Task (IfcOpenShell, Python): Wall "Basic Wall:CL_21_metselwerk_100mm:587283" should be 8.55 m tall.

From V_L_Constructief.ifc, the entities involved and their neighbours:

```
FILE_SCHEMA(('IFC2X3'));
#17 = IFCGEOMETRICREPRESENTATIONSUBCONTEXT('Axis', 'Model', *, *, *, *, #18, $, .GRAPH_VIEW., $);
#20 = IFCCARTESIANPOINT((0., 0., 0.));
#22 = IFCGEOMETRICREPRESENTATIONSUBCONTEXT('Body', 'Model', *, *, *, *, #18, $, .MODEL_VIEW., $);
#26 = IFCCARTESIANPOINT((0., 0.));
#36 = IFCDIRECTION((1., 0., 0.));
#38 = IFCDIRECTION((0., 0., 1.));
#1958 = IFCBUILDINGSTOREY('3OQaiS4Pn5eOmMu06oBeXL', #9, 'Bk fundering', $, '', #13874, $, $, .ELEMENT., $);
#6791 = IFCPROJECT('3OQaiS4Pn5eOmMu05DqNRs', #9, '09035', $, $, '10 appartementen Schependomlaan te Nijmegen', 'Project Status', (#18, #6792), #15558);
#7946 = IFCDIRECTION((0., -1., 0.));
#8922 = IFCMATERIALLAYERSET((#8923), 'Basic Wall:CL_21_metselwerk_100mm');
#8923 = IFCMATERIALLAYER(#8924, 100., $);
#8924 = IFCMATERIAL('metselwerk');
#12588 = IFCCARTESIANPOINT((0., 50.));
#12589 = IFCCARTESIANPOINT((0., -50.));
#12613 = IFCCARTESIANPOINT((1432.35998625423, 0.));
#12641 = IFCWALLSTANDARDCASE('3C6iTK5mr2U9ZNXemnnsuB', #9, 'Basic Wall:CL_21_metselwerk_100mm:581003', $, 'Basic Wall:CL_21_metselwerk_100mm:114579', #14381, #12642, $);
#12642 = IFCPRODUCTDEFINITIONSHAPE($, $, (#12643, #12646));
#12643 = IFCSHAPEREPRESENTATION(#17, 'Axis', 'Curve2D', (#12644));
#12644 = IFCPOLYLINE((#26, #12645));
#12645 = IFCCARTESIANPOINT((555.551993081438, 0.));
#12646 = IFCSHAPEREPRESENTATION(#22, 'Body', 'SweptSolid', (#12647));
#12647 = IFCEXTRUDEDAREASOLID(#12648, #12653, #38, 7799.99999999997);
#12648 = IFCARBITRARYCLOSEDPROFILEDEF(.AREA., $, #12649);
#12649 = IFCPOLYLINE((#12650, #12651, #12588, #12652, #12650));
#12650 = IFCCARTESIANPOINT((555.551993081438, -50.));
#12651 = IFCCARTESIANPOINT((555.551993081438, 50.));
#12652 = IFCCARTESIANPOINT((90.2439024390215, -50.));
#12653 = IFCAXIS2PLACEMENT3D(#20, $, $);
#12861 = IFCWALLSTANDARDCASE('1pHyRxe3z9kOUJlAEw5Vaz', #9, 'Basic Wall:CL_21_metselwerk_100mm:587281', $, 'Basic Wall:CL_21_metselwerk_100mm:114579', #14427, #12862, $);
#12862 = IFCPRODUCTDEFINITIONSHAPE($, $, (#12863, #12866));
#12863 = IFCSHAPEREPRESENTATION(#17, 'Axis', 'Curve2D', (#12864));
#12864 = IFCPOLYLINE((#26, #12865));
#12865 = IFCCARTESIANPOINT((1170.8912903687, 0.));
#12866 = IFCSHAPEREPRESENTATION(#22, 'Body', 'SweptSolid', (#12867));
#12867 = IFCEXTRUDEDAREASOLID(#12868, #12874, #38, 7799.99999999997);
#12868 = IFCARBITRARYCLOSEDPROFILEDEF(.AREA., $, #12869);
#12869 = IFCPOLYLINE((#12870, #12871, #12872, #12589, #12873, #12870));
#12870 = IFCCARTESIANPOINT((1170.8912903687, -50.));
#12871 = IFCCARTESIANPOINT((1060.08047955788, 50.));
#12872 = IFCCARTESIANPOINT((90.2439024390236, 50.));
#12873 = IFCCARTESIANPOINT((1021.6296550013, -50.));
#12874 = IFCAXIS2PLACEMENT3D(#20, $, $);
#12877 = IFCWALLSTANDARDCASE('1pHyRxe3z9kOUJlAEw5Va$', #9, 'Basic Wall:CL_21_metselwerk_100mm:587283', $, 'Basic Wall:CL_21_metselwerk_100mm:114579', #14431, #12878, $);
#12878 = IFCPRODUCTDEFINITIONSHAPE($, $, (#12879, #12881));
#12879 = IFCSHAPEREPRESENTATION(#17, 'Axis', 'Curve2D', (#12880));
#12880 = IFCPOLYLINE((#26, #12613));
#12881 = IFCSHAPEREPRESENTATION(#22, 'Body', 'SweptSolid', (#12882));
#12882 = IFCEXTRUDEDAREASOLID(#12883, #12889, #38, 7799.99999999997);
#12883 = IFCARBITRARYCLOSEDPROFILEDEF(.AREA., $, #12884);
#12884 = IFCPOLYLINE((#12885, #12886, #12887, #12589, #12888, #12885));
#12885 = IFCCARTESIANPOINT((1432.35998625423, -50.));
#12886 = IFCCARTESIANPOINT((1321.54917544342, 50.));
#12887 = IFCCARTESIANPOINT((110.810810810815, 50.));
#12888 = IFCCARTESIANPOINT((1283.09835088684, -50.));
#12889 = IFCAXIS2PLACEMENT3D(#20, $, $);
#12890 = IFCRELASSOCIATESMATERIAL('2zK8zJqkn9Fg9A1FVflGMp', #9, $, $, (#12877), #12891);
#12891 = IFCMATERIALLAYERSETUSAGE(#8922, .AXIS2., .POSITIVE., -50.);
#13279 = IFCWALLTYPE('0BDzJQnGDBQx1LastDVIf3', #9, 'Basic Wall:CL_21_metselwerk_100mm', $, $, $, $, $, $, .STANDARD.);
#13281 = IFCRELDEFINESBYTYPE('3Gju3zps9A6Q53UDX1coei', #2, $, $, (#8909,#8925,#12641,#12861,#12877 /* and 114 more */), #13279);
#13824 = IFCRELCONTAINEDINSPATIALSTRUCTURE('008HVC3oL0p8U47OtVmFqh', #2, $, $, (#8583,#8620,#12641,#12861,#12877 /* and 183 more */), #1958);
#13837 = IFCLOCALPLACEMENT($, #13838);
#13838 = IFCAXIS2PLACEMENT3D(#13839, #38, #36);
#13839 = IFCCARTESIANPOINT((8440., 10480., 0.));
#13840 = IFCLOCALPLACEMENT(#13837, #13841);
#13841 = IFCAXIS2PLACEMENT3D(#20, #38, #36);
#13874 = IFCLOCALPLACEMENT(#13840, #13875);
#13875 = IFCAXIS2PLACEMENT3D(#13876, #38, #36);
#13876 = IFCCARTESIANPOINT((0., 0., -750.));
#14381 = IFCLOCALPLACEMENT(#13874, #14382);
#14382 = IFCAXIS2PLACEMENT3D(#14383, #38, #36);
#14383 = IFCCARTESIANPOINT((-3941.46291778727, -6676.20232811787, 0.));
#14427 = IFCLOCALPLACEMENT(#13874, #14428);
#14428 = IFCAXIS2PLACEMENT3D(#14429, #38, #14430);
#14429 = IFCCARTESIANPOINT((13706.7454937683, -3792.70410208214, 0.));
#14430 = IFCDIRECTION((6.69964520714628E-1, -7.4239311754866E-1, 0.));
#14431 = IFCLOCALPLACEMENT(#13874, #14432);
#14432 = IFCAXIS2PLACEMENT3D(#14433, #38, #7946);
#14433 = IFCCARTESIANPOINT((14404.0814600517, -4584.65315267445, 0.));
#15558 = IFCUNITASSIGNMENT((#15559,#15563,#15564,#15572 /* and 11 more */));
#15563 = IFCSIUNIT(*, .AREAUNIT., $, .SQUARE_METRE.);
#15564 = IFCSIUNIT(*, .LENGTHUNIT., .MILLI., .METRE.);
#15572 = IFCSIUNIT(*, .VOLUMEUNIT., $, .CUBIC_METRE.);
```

```python
import ifcopenshell
import ifcopenshell.geom
import ifcopenshell.util.representation
import ifcopenshell.util.shape

model = ifcopenshell.open("V_L_Constructief.ifc")
settings = ifcopenshell.geom.settings()


def volume(element):
    """Net volume in cubic metres, openings subtracted."""
    shape = ifcopenshell.geom.create_shape(settings, element)
    return ifcopenshell.util.shape.get_volume(shape.geometry)


wall = model.by_guid("1pHyRxe3z9kOUJlAEw5Va$")
before = volume(wall)

body = ifcopenshell.util.representation.get_representation(wall, "Model", "Body")
solid = body.Items[0]
old_height = solid.Depth
solid.Depth = 8550.0
after = volume(wall)

print(f"height {old_height:g} -> {solid.Depth:g}, volume {before:.3f} -> {after:.3f} m3")

model.write("V_L_Constructief_updated.ifc")
```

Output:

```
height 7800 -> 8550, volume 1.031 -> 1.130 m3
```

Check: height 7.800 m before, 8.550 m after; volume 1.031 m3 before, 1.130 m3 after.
